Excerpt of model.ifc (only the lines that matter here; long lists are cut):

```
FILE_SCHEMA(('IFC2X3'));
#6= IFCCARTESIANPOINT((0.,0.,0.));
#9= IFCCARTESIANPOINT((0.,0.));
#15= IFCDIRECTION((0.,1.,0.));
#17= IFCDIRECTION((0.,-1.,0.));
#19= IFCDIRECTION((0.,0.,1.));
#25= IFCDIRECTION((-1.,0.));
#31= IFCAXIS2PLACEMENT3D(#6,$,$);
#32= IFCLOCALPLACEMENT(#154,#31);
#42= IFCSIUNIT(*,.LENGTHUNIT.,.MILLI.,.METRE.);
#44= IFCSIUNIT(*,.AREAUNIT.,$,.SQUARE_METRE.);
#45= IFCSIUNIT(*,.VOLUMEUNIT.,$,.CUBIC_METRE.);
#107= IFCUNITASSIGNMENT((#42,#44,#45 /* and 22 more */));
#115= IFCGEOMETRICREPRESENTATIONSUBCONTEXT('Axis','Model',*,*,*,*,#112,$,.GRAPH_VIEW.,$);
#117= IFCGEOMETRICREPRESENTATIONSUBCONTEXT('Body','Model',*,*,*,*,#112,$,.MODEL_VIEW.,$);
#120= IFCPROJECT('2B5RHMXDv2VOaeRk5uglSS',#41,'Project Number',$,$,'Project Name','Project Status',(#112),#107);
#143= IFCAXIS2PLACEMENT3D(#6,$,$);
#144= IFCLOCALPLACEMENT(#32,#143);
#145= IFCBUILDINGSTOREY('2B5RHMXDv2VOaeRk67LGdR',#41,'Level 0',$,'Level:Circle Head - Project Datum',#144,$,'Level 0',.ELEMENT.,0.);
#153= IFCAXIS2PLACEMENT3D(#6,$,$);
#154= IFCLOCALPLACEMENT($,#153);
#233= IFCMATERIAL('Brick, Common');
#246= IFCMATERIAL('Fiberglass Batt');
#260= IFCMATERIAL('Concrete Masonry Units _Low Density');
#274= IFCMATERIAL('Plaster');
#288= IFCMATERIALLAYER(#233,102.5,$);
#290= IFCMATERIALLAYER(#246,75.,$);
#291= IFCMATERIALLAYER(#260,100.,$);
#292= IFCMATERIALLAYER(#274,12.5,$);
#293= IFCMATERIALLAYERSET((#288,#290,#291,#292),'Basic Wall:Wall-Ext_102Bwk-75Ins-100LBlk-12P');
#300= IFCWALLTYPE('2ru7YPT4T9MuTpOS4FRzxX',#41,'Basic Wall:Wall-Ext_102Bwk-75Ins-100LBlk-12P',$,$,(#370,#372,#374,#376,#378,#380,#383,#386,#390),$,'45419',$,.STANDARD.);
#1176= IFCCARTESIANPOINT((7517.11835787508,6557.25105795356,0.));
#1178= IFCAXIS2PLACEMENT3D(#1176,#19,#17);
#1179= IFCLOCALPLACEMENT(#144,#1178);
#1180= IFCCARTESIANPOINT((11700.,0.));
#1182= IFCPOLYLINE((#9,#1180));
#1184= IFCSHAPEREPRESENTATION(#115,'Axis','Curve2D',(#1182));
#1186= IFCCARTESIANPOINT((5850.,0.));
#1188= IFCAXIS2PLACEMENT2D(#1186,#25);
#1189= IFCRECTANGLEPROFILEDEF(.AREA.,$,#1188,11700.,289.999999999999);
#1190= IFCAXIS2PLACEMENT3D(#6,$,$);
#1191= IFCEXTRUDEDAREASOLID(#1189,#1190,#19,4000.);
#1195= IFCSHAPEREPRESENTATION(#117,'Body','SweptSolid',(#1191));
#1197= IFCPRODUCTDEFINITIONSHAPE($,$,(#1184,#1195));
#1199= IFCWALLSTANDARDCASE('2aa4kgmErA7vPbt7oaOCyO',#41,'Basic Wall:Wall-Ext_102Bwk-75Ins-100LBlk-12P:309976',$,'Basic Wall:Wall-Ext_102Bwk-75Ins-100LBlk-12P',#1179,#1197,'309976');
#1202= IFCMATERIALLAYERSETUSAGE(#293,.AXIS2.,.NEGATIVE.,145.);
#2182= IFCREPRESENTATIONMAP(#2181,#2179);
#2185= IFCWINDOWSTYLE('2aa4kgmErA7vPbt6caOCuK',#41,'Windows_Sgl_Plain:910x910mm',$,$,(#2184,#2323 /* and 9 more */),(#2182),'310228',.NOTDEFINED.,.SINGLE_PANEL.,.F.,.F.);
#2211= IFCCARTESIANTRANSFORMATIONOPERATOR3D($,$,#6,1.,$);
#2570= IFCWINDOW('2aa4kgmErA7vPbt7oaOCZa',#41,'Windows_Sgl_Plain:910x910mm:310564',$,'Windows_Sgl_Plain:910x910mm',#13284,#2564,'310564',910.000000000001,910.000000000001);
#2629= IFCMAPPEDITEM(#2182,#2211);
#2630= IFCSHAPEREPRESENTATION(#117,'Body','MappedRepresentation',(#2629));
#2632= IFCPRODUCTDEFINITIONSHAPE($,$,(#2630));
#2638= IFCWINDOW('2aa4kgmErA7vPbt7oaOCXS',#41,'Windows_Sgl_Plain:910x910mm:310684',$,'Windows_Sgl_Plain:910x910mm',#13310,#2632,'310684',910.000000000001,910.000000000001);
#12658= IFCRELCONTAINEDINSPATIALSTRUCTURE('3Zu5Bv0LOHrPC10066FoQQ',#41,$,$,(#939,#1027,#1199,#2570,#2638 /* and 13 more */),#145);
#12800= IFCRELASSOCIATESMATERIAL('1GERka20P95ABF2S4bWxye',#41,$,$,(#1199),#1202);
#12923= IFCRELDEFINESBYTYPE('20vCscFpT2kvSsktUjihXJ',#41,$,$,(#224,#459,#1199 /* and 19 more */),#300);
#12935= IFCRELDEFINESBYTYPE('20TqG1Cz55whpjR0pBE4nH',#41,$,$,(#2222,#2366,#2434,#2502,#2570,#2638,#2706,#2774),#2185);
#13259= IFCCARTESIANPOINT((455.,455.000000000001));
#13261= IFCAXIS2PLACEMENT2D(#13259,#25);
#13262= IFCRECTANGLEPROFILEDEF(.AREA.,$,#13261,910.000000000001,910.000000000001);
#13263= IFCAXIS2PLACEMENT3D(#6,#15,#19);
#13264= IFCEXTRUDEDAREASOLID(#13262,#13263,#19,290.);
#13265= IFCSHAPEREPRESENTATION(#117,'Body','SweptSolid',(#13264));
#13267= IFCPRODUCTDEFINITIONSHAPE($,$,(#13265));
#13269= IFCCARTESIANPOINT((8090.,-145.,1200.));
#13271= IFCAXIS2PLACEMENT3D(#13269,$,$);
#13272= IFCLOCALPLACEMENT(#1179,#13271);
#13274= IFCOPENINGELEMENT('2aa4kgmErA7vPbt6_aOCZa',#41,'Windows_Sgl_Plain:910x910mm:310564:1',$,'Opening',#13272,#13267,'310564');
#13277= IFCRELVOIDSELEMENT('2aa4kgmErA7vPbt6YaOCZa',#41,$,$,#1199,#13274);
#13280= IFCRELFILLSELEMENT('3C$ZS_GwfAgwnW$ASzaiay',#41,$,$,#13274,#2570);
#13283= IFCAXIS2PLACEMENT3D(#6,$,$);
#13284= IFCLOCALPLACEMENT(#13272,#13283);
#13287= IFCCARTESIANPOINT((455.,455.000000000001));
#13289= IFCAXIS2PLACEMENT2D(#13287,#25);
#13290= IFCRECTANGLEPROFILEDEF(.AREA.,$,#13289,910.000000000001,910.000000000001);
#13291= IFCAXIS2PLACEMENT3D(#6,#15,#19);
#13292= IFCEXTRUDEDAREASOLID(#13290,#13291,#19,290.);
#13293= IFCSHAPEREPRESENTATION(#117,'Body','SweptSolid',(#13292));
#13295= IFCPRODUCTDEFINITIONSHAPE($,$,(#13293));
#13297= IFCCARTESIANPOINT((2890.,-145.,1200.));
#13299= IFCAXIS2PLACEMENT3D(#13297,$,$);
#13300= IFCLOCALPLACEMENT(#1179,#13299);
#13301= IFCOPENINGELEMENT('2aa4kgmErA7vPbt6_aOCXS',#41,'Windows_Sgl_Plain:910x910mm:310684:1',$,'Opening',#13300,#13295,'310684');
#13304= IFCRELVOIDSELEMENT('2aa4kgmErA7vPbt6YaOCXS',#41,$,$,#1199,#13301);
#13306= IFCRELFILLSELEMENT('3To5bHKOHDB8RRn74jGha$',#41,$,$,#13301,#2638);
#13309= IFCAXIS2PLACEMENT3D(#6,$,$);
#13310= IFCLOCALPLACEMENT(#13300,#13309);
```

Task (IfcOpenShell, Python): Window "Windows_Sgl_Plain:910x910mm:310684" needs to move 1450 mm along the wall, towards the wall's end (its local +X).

```python
import ifcopenshell
import ifcopenshell.api.geometry
import ifcopenshell.util.placement

model = ifcopenshell.open("model.ifc")

window = model.by_guid("2aa4kgmErA7vPbt7oaOCXS")
opening = window.FillsVoids[0].RelatingOpeningElement
wall = opening.VoidsElements[0].RelatingBuildingElement

wall_matrix = ifcopenshell.util.placement.get_local_placement(wall.ObjectPlacement)
shift = wall_matrix[:3, 0] * 1450.0
before = ifcopenshell.util.placement.get_local_placement(window.ObjectPlacement)[:3, 3].copy()

# The window is placed relative to its opening, so it follows when the opening moves.
matrix = ifcopenshell.util.placement.get_local_placement(opening.ObjectPlacement)
matrix[:3, 3] += shift
ifcopenshell.api.geometry.edit_object_placement(
    model, product=opening, matrix=matrix, is_si=False, should_transform_children=True
)

after = ifcopenshell.util.placement.get_local_placement(window.ObjectPlacement)[:3, 3]
print("window moved by", (after - before).round(3) + 0.0)

model.write("model_v2.ifc")
```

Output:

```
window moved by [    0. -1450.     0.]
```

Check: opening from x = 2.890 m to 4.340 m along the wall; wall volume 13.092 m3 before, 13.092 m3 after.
